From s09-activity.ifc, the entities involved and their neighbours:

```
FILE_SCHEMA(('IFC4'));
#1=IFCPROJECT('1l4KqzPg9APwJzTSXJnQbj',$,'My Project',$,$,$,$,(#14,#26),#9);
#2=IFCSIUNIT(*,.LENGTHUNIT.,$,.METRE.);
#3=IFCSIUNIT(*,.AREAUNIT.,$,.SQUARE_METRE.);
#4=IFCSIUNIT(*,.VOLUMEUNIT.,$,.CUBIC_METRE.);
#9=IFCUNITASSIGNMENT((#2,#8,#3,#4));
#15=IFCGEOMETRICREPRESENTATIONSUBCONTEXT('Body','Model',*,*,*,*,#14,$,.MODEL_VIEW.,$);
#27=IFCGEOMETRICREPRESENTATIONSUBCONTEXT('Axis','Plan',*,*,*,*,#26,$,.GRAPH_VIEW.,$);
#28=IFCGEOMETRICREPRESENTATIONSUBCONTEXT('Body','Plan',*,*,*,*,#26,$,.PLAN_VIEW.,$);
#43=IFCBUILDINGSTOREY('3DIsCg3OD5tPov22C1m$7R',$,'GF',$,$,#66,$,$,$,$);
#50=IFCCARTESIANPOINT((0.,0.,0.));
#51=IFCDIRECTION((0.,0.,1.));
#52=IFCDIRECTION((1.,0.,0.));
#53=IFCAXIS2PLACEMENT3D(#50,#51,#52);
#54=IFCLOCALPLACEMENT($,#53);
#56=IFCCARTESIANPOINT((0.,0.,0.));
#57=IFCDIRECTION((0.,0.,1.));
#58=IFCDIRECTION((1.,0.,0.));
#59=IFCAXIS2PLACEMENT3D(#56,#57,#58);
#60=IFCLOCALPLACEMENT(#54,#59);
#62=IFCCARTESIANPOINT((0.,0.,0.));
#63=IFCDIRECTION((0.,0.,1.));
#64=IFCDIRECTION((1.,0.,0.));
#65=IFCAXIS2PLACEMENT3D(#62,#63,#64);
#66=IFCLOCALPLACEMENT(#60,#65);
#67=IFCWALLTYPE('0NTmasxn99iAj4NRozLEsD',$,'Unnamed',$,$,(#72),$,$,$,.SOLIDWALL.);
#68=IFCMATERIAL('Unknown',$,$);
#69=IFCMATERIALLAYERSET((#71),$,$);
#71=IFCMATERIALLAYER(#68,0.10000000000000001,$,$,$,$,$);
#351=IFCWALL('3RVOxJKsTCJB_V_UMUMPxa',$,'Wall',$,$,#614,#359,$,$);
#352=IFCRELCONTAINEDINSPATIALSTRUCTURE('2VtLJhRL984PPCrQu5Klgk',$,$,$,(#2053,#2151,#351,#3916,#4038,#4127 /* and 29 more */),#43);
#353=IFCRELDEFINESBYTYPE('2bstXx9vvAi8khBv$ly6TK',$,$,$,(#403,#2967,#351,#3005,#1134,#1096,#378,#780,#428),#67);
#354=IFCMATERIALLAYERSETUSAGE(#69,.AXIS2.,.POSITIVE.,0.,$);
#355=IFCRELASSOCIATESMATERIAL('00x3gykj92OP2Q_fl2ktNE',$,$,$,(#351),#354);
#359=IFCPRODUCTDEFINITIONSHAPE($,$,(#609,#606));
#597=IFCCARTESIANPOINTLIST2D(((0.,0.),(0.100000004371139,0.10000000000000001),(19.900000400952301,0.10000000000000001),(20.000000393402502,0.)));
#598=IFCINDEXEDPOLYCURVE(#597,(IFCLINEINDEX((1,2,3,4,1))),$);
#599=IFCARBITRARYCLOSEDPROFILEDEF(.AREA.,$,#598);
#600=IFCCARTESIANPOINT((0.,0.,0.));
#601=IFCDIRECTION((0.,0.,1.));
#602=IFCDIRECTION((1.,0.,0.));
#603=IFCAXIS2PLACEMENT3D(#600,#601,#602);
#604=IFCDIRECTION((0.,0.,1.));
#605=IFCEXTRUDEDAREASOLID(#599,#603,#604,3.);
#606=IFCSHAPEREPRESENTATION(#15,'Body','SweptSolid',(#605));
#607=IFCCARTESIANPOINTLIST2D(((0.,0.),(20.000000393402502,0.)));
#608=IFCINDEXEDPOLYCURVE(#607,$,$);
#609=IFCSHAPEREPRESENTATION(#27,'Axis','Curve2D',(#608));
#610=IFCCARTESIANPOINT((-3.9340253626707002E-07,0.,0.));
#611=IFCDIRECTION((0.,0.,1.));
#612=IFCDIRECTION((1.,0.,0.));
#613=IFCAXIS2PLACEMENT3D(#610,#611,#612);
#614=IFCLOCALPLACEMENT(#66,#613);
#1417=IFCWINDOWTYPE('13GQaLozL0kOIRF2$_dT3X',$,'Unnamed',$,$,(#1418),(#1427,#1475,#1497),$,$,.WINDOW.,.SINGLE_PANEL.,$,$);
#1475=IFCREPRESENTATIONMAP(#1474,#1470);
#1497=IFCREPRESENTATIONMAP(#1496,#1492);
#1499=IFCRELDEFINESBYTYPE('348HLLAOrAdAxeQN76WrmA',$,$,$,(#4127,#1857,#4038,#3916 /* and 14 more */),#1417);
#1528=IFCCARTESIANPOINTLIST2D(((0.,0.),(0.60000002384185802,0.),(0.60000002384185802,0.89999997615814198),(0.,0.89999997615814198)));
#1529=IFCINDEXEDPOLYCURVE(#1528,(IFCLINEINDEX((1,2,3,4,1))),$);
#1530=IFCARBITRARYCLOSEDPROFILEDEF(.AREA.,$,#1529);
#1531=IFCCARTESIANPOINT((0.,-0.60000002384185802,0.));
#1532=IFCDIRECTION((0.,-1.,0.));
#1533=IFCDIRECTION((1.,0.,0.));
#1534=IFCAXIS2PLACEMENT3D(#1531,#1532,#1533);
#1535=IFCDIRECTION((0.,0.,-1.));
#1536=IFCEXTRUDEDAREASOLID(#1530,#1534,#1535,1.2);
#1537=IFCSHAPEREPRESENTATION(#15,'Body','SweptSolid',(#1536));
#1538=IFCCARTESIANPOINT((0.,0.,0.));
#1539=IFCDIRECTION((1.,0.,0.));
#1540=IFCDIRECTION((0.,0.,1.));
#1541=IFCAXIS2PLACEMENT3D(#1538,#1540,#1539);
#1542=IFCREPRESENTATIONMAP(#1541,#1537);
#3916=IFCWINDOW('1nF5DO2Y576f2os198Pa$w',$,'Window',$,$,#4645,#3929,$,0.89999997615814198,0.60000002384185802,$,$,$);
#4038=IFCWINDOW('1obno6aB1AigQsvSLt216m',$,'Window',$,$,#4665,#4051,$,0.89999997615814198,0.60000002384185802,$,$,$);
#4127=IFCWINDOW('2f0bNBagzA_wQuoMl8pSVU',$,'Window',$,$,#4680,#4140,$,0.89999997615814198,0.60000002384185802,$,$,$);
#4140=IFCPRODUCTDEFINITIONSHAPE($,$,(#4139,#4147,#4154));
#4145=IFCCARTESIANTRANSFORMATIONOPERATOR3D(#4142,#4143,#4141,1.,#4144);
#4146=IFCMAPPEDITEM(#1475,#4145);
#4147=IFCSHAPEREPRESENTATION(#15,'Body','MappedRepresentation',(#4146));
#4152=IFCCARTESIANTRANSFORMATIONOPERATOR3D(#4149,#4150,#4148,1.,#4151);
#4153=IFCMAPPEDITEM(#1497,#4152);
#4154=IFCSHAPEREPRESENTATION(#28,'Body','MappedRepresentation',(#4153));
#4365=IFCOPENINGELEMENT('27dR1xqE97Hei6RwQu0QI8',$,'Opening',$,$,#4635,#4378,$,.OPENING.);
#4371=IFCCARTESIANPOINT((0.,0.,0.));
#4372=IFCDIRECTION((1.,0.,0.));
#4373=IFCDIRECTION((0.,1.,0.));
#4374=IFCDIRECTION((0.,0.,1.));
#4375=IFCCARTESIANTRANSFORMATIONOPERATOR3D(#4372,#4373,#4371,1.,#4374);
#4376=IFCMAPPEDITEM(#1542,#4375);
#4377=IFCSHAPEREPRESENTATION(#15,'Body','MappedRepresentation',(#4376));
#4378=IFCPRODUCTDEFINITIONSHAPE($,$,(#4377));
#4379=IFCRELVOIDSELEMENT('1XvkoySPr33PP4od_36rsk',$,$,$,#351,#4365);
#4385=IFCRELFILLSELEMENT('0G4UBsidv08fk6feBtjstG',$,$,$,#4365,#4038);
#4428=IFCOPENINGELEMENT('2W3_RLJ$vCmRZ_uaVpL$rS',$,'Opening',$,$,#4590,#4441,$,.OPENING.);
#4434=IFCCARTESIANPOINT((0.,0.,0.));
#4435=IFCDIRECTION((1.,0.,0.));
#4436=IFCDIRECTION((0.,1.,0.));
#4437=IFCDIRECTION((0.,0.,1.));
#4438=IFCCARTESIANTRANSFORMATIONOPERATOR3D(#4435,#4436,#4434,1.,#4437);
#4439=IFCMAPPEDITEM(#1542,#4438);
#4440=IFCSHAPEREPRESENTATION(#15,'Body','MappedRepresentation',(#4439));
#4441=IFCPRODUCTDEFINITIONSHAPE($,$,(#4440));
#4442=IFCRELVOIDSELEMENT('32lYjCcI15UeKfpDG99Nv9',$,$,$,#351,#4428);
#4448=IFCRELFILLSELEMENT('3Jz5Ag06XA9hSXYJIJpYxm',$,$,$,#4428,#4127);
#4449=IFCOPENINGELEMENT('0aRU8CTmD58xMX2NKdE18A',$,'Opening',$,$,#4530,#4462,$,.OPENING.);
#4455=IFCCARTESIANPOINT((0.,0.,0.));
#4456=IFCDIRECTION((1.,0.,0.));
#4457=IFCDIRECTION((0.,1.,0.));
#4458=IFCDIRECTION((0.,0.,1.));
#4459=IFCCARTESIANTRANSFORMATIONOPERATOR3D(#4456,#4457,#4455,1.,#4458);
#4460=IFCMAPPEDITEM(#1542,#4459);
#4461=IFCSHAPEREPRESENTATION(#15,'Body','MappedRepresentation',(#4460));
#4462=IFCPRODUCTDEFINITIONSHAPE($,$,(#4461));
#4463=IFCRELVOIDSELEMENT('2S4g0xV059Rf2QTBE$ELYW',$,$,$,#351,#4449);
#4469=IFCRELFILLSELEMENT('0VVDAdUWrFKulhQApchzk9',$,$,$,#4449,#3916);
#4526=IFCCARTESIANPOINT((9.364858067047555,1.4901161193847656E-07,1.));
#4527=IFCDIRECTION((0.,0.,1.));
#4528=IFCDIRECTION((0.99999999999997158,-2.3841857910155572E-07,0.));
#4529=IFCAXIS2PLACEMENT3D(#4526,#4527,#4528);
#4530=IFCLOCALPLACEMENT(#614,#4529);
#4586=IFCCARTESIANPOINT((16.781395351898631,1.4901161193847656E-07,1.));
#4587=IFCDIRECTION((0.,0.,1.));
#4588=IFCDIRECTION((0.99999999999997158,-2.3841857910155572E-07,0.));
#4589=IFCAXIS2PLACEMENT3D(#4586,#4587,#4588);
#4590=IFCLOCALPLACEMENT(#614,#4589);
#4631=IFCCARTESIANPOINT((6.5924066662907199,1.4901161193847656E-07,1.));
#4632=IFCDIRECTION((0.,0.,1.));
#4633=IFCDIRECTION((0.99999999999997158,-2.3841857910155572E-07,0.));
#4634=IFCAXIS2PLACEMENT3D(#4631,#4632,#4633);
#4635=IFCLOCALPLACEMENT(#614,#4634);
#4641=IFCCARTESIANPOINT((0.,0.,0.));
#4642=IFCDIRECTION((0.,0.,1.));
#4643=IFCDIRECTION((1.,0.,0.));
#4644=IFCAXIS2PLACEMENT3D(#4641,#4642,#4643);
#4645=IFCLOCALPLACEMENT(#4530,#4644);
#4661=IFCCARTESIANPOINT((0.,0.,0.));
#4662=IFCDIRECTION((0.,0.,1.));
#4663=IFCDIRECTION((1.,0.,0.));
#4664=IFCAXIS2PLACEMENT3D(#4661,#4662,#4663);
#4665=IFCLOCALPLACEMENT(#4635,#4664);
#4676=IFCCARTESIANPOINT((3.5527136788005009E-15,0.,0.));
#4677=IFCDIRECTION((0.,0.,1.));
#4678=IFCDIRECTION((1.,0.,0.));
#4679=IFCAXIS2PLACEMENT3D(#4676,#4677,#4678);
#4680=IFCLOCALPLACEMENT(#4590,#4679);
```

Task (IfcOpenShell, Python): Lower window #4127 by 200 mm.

```python
import numpy as np
import ifcopenshell
import ifcopenshell.api.geometry
import ifcopenshell.util.placement
import ifcopenshell.util.unit

model = ifcopenshell.open("s09-activity.ifc")
unit_scale = ifcopenshell.util.unit.calculate_unit_scale(model)

window = model.by_guid("2f0bNBagzA_wQuoMl8pSVU")
opening = window.FillsVoids[0].RelatingOpeningElement
dz = -0.2 / unit_scale

shift = np.array([0.0, 0.0, dz])
# The window is placed relative to its opening, so it follows when the opening moves.
matrix = ifcopenshell.util.placement.get_local_placement(opening.ObjectPlacement)
matrix[:3, 3] += shift
ifcopenshell.api.geometry.edit_object_placement(
    model, product=opening, matrix=matrix, is_si=False, should_transform_children=True
)

print(f"moved by {dz * unit_scale:+.3f} m")

model.write("s09-activity-out.ifc")
```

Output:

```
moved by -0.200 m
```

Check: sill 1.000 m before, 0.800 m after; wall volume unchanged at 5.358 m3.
